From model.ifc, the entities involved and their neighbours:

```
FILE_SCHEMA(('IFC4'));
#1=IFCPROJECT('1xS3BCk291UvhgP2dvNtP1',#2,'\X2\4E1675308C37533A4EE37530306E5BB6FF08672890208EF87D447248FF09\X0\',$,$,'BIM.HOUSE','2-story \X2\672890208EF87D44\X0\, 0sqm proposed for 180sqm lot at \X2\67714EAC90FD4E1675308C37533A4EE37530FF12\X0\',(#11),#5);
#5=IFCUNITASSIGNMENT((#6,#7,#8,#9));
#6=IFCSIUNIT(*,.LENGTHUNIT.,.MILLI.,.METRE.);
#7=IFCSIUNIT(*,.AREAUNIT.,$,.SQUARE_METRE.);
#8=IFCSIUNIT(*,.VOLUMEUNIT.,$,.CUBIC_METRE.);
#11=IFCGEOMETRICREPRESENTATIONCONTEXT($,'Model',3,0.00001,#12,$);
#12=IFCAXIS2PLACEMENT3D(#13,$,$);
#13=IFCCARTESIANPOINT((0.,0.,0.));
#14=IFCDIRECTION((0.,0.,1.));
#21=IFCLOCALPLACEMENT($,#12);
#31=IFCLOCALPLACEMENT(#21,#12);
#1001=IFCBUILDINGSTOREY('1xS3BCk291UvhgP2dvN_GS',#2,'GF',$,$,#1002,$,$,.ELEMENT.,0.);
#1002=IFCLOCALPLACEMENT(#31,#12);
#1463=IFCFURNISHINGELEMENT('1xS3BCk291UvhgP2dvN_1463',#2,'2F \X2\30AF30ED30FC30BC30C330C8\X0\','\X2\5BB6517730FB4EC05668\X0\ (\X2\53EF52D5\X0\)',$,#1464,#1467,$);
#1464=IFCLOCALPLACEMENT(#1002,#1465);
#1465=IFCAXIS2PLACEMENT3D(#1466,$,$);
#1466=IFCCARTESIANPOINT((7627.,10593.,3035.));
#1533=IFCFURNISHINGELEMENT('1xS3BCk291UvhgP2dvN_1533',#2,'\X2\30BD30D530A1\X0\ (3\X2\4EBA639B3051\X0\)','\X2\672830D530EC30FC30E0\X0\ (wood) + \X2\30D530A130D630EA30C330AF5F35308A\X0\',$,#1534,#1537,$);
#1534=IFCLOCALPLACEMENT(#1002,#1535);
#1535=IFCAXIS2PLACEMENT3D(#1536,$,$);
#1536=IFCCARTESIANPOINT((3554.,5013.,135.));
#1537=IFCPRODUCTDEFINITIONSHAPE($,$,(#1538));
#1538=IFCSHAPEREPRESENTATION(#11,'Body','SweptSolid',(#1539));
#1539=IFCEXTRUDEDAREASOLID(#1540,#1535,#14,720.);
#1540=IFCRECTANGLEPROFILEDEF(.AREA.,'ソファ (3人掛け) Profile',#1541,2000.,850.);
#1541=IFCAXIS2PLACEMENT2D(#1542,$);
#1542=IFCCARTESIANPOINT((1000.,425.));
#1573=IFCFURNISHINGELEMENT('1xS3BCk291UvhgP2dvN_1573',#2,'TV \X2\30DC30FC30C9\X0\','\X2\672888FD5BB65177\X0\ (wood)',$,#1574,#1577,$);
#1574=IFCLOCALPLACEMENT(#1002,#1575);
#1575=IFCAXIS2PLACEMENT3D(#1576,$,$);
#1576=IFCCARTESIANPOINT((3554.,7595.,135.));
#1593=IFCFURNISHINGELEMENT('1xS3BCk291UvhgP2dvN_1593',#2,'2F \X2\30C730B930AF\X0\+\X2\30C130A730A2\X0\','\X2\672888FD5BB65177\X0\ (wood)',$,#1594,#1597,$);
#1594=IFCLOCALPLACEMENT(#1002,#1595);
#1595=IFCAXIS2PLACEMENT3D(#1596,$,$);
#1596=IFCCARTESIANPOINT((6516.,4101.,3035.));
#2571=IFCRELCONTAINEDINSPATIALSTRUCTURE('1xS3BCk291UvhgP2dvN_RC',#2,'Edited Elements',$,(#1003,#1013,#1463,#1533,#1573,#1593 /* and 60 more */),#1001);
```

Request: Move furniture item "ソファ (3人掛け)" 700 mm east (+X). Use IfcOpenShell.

```python
import ifcopenshell
import ifcopenshell.api.geometry
import ifcopenshell.util.placement

model = ifcopenshell.open("model.ifc")

item = model.by_id(1533)
matrix = ifcopenshell.util.placement.get_local_placement(item.ObjectPlacement)
matrix[0, 3] += 700.0
ifcopenshell.api.geometry.edit_object_placement(model, product=item, matrix=matrix, is_si=False)

print(ifcopenshell.util.placement.get_local_placement(item.ObjectPlacement).round(3) + 0.0)

model.write("model_updated.ifc")
```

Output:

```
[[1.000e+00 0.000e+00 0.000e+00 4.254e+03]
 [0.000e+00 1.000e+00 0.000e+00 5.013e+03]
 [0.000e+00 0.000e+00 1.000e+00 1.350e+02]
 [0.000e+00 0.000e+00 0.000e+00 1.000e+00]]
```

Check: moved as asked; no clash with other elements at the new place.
